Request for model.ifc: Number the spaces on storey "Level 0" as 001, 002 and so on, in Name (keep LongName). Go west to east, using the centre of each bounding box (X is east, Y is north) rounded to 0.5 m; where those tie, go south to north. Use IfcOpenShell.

First a look at what the model holds.

```python
import ifcopenshell
import ifcopenshell.util.element
import ifcopenshell.util.placement

model = ifcopenshell.open("model.ifc")
print(model.schema)
storey = next(s for s in model.by_type("IfcBuildingStorey") if s.Name == "Level 0")
spaces = [e for e in ifcopenshell.util.element.get_decomposition(storey) if e.is_a("IfcSpace")]
for e in sorted(spaces, key=lambda e: e.id()):
    origin = ifcopenshell.util.placement.get_local_placement(e.ObjectPlacement)[:3, 3]
    print(e.id(), e.Name, e.LongName, origin.round(2) + 0.0, sep=" | ")
```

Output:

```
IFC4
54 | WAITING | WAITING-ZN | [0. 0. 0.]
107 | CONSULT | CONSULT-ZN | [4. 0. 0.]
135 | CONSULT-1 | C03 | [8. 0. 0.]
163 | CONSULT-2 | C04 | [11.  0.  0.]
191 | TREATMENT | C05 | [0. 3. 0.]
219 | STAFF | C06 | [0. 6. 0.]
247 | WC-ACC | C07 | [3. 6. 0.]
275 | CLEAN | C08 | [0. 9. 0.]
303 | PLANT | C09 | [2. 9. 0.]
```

```python
import ifcopenshell
import ifcopenshell.geom
import ifcopenshell.util.element
import ifcopenshell.util.shape

model = ifcopenshell.open("model.ifc")
settings = ifcopenshell.geom.settings()
settings.set("use-world-coords", True)


def centre(element):
    shape = ifcopenshell.geom.create_shape(settings, element)
    return ifcopenshell.util.shape.get_bbox_centroid(shape.geometry)


storey = next(s for s in model.by_type("IfcBuildingStorey") if s.Name == "Level 0")
spaces = [e for e in ifcopenshell.util.element.get_decomposition(storey) if e.is_a("IfcSpace")]

# Insertion points can sit at a corner or the storey origin, so sort by the geometry (in metres).
centres = {e: centre(e) for e in spaces}
spaces.sort(key=lambda e: (round(centres[e][0] / 0.5), centres[e][1]))

for i, e in enumerate(spaces, start=1):
    number = f"0{i:02d}"
    e.Name = number
    print(e.id(), number)

model.write("model_rev.ifc")
```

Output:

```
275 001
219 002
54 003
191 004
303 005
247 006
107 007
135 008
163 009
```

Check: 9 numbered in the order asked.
